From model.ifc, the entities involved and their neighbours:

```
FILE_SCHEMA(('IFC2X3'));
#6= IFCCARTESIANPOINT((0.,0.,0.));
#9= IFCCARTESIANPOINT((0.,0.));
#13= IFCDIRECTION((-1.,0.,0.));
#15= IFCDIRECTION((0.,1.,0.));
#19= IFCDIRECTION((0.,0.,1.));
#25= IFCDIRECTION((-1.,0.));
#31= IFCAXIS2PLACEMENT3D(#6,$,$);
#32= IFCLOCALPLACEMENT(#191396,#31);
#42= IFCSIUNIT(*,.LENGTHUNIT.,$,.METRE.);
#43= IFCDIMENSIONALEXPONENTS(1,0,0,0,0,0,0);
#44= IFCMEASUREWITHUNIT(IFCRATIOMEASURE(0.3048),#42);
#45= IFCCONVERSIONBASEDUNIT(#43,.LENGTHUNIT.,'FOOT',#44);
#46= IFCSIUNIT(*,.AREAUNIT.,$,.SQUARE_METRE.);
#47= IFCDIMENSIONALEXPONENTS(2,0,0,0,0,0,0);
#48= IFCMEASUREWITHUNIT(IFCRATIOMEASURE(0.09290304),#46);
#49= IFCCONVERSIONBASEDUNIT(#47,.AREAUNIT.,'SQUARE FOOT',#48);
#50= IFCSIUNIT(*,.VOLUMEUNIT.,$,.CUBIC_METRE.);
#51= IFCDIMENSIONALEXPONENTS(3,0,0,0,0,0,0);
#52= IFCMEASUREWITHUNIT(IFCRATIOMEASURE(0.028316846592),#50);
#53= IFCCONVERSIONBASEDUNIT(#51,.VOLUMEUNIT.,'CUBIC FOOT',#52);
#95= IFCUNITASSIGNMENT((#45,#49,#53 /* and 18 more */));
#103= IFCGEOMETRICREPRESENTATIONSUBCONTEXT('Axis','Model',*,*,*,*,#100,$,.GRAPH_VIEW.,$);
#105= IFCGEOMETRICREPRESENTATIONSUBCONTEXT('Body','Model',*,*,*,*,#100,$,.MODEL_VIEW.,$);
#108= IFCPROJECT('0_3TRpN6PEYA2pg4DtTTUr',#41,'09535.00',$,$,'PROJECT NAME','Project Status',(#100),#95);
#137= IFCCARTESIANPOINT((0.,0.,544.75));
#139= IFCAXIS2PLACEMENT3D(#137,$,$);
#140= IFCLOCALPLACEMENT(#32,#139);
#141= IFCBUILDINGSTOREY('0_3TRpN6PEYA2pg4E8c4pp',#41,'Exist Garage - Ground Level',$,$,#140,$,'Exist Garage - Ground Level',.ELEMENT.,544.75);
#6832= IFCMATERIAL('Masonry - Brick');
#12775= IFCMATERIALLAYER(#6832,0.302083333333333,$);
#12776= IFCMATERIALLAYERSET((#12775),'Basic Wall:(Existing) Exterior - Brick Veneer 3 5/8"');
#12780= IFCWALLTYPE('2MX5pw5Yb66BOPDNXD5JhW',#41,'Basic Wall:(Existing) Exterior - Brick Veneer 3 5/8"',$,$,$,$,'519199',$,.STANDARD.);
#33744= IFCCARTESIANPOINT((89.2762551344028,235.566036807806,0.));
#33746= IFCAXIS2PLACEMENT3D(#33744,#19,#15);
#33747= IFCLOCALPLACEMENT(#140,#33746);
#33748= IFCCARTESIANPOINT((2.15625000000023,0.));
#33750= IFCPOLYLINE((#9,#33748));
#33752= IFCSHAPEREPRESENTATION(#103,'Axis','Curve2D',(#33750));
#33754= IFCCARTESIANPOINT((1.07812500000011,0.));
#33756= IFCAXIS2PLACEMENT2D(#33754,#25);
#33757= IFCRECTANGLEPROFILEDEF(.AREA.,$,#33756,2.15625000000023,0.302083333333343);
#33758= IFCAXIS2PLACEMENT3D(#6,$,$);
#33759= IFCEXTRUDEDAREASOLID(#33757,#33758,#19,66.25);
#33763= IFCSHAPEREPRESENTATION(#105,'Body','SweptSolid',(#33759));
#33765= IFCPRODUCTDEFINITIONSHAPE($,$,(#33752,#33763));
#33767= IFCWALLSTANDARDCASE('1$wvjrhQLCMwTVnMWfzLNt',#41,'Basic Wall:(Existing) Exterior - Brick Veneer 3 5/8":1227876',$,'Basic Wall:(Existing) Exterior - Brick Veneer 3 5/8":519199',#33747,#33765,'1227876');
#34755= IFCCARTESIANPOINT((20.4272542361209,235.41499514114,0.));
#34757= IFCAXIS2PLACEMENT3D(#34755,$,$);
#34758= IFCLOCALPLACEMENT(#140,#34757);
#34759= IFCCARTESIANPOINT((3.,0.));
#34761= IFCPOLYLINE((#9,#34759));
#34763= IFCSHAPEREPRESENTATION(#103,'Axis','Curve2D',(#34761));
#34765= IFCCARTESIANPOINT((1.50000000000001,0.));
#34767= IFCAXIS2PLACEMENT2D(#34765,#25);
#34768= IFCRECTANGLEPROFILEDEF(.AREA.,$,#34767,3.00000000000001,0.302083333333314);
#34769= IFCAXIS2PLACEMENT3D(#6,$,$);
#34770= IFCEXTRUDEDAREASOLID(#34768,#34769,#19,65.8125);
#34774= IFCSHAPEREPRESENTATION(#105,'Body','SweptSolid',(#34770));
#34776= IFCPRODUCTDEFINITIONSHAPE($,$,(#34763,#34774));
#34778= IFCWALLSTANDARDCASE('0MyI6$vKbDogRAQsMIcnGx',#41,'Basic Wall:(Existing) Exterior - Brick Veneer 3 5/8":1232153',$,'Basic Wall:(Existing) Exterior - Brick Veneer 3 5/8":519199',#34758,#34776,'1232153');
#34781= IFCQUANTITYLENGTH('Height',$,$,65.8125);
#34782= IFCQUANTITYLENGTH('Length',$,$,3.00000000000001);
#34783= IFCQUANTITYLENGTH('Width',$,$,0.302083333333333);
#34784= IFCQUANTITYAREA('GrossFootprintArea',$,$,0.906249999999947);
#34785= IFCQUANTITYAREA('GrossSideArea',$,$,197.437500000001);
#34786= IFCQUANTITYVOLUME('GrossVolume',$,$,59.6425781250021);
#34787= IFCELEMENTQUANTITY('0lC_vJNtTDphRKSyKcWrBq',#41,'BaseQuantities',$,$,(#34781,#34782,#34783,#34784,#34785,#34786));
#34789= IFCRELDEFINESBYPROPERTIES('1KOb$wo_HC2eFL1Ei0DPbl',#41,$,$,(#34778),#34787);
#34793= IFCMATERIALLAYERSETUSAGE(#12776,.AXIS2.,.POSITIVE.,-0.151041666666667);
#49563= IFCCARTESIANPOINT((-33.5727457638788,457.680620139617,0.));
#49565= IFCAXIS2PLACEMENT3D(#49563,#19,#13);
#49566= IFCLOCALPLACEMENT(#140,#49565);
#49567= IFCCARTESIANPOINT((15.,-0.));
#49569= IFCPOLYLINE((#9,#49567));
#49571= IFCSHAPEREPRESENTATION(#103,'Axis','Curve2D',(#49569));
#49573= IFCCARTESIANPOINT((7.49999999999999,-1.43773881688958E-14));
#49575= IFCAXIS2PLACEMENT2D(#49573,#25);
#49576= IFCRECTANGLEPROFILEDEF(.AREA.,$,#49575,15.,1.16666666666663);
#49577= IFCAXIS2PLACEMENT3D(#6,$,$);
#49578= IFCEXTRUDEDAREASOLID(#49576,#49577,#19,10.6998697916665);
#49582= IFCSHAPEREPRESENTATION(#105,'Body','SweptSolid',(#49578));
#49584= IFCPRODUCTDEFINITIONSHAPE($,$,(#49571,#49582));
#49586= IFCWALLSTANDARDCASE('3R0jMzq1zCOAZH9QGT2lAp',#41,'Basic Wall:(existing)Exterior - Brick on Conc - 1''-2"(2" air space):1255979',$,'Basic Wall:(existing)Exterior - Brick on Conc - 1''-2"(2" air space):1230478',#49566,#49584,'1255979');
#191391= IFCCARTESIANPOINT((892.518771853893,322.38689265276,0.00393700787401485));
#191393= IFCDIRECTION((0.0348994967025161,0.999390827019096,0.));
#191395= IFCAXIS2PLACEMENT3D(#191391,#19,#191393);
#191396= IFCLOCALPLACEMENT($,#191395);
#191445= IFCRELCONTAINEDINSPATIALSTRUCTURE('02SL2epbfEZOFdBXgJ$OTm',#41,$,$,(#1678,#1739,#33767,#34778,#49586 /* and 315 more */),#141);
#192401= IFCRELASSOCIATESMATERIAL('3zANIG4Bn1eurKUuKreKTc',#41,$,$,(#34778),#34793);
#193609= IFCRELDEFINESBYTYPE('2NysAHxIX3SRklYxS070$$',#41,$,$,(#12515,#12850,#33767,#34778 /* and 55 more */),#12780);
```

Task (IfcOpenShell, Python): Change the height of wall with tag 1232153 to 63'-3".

```python
import ifcopenshell
import ifcopenshell.api.pset
import ifcopenshell.geom
import ifcopenshell.util.element
import ifcopenshell.util.representation
import ifcopenshell.util.shape
import ifcopenshell.util.unit

model = ifcopenshell.open("model.ifc")
unit_scale = ifcopenshell.util.unit.calculate_unit_scale(model)
area_scale = ifcopenshell.util.unit.calculate_unit_scale(model, "AREAUNIT")
volume_scale = ifcopenshell.util.unit.calculate_unit_scale(model, "VOLUMEUNIT")
settings = ifcopenshell.geom.settings()


def volume(element):
    """Net volume in cubic metres, openings subtracted."""
    shape = ifcopenshell.geom.create_shape(settings, element)
    return ifcopenshell.util.shape.get_volume(shape.geometry)


wall = model.by_id(34778)
before = volume(wall)

body = ifcopenshell.util.representation.get_representation(wall, "Model", "Body")
solid = body.Items[0]
old_height = solid.Depth
solid.Depth = 759 * 0.0254 / unit_scale
after = volume(wall)

# Update the stored height, areas and volumes.
qto = model.by_id(ifcopenshell.util.element.get_pset(wall, "BaseQuantities", should_inherit=False)["id"])
ifcopenshell.api.pset.edit_qto(model, qto=qto, properties={
    "Height": solid.Depth,
    "GrossSideArea": ifcopenshell.util.element.get_pset(wall, "BaseQuantities", "GrossSideArea") * solid.Depth / old_height,
    "GrossVolume": ifcopenshell.util.element.get_pset(wall, "BaseQuantities", "GrossVolume") * solid.Depth / old_height,
})

print(f"height {old_height:g} -> {solid.Depth:g}, volume {before:.3f} -> {after:.3f} m3")

model.write("model_v2.ifc")
```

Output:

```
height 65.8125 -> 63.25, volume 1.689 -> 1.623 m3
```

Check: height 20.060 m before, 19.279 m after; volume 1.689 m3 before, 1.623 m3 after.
